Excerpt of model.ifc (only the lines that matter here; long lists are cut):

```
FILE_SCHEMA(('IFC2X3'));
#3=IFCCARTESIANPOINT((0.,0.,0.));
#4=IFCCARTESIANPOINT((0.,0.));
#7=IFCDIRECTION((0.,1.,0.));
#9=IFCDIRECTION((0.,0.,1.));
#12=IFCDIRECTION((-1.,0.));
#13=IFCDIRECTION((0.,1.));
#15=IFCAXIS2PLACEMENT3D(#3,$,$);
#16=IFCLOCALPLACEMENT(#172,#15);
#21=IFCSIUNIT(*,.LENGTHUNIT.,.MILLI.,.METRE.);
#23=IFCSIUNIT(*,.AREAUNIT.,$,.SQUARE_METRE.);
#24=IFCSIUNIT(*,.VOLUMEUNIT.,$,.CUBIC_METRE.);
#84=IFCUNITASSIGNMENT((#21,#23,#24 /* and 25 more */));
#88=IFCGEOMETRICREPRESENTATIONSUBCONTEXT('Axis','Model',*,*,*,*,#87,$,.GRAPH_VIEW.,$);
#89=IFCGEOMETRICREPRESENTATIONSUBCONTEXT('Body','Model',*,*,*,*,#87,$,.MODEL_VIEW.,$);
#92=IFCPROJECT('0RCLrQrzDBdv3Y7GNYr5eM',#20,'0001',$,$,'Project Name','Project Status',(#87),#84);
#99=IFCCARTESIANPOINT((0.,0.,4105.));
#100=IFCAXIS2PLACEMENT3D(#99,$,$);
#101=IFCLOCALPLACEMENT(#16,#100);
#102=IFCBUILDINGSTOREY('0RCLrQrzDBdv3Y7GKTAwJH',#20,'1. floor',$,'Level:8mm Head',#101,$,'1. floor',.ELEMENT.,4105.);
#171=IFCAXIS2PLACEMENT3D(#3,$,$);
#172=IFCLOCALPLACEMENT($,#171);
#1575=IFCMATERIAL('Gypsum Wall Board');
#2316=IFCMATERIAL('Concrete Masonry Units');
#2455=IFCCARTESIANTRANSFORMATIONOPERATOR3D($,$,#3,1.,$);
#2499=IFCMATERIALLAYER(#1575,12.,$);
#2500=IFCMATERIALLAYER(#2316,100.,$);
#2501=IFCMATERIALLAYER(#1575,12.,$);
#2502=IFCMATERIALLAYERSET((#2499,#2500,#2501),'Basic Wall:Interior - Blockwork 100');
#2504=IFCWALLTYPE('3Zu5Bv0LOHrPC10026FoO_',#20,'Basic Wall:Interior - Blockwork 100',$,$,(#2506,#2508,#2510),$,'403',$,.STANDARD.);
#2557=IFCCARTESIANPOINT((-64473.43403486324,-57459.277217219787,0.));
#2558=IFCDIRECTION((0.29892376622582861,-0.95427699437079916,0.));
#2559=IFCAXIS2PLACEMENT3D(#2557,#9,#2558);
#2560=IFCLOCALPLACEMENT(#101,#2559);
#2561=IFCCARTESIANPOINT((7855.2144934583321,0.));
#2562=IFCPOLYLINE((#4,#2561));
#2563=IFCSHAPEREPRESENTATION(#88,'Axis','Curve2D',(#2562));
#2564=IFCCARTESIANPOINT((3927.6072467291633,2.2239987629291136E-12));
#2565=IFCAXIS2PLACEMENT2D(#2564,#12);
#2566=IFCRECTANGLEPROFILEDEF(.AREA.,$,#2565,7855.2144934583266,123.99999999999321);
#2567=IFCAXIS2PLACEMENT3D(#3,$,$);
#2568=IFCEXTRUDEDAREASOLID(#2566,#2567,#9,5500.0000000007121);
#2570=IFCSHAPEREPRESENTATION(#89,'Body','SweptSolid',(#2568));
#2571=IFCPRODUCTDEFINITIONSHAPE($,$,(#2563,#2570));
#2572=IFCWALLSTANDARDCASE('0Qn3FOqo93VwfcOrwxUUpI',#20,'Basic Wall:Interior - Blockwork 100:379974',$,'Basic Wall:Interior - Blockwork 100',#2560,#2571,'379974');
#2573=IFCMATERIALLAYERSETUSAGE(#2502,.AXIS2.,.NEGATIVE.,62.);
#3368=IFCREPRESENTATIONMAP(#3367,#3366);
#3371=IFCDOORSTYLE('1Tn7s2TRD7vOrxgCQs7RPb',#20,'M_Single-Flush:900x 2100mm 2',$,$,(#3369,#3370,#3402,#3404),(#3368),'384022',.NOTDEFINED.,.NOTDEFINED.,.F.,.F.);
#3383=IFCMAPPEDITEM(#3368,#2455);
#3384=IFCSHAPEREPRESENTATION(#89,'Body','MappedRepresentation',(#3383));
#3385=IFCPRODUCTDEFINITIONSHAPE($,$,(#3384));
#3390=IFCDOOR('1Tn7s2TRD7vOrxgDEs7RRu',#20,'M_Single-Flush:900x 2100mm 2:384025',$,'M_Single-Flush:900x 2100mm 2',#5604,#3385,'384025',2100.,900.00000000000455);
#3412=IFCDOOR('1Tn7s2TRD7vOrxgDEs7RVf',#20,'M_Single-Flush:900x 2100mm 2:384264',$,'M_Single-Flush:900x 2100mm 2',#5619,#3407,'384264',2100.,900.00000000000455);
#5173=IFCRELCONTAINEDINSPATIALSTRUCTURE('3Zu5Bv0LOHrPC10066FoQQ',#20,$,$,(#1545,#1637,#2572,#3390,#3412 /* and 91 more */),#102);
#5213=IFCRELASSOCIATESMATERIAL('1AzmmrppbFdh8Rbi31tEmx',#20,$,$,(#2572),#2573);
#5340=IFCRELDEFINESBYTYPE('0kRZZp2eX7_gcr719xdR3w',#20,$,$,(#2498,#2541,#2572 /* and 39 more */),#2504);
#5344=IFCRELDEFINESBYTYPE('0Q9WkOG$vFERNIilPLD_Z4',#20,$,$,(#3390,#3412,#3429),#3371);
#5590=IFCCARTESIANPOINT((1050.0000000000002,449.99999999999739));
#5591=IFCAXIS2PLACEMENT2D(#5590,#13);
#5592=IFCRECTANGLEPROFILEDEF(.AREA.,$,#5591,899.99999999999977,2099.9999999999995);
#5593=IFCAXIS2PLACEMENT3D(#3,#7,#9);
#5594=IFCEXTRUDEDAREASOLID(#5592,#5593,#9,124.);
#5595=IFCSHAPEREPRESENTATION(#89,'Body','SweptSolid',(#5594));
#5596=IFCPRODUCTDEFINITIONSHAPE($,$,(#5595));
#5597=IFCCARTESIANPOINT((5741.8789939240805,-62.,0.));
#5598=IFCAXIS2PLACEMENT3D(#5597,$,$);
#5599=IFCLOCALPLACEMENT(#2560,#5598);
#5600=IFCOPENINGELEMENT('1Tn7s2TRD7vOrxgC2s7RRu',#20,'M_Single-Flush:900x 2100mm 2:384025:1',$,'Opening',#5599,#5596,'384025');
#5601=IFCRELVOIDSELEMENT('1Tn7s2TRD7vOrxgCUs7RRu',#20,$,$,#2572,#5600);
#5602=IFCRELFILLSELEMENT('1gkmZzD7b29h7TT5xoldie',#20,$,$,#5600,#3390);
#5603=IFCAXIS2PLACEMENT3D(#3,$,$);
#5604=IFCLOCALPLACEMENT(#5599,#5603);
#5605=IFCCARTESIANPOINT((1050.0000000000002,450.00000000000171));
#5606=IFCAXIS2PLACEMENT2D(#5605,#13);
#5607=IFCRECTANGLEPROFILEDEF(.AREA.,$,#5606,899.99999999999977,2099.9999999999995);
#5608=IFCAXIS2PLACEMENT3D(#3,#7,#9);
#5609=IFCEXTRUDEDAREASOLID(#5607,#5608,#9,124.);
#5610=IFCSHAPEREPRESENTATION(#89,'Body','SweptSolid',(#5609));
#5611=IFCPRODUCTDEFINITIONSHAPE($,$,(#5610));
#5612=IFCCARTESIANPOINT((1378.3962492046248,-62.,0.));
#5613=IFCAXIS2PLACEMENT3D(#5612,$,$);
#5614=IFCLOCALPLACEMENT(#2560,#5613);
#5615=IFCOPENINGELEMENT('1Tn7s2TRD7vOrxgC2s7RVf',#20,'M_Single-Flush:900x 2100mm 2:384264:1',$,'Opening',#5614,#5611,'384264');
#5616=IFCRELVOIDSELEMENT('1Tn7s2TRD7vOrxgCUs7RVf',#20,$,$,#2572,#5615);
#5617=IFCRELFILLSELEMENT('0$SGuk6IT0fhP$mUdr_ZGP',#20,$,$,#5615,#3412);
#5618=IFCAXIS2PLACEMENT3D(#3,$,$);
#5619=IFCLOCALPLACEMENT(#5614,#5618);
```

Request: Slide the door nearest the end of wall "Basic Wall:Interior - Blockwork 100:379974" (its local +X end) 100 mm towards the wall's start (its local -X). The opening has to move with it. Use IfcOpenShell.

```python
import ifcopenshell
import ifcopenshell.api.geometry
import ifcopenshell.util.placement

model = ifcopenshell.open("model.ifc")

door = model.by_guid("1Tn7s2TRD7vOrxgDEs7RRu")
opening = door.FillsVoids[0].RelatingOpeningElement
wall = opening.VoidsElements[0].RelatingBuildingElement

wall_matrix = ifcopenshell.util.placement.get_local_placement(wall.ObjectPlacement)
shift = wall_matrix[:3, 0] * -100.0
before = ifcopenshell.util.placement.get_local_placement(door.ObjectPlacement)[:3, 3].copy()

# The door is placed relative to its opening, so it follows when the opening moves.
matrix = ifcopenshell.util.placement.get_local_placement(opening.ObjectPlacement)
matrix[:3, 3] += shift
ifcopenshell.api.geometry.edit_object_placement(
    model, product=opening, matrix=matrix, is_si=False, should_transform_children=True
)

after = ifcopenshell.util.placement.get_local_placement(door.ObjectPlacement)[:3, 3]
print("door moved by", (after - before).round(3) + 0.0)

model.write("model-out.ifc")
```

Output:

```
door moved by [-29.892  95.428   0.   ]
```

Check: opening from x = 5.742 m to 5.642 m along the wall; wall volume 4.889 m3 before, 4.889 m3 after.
